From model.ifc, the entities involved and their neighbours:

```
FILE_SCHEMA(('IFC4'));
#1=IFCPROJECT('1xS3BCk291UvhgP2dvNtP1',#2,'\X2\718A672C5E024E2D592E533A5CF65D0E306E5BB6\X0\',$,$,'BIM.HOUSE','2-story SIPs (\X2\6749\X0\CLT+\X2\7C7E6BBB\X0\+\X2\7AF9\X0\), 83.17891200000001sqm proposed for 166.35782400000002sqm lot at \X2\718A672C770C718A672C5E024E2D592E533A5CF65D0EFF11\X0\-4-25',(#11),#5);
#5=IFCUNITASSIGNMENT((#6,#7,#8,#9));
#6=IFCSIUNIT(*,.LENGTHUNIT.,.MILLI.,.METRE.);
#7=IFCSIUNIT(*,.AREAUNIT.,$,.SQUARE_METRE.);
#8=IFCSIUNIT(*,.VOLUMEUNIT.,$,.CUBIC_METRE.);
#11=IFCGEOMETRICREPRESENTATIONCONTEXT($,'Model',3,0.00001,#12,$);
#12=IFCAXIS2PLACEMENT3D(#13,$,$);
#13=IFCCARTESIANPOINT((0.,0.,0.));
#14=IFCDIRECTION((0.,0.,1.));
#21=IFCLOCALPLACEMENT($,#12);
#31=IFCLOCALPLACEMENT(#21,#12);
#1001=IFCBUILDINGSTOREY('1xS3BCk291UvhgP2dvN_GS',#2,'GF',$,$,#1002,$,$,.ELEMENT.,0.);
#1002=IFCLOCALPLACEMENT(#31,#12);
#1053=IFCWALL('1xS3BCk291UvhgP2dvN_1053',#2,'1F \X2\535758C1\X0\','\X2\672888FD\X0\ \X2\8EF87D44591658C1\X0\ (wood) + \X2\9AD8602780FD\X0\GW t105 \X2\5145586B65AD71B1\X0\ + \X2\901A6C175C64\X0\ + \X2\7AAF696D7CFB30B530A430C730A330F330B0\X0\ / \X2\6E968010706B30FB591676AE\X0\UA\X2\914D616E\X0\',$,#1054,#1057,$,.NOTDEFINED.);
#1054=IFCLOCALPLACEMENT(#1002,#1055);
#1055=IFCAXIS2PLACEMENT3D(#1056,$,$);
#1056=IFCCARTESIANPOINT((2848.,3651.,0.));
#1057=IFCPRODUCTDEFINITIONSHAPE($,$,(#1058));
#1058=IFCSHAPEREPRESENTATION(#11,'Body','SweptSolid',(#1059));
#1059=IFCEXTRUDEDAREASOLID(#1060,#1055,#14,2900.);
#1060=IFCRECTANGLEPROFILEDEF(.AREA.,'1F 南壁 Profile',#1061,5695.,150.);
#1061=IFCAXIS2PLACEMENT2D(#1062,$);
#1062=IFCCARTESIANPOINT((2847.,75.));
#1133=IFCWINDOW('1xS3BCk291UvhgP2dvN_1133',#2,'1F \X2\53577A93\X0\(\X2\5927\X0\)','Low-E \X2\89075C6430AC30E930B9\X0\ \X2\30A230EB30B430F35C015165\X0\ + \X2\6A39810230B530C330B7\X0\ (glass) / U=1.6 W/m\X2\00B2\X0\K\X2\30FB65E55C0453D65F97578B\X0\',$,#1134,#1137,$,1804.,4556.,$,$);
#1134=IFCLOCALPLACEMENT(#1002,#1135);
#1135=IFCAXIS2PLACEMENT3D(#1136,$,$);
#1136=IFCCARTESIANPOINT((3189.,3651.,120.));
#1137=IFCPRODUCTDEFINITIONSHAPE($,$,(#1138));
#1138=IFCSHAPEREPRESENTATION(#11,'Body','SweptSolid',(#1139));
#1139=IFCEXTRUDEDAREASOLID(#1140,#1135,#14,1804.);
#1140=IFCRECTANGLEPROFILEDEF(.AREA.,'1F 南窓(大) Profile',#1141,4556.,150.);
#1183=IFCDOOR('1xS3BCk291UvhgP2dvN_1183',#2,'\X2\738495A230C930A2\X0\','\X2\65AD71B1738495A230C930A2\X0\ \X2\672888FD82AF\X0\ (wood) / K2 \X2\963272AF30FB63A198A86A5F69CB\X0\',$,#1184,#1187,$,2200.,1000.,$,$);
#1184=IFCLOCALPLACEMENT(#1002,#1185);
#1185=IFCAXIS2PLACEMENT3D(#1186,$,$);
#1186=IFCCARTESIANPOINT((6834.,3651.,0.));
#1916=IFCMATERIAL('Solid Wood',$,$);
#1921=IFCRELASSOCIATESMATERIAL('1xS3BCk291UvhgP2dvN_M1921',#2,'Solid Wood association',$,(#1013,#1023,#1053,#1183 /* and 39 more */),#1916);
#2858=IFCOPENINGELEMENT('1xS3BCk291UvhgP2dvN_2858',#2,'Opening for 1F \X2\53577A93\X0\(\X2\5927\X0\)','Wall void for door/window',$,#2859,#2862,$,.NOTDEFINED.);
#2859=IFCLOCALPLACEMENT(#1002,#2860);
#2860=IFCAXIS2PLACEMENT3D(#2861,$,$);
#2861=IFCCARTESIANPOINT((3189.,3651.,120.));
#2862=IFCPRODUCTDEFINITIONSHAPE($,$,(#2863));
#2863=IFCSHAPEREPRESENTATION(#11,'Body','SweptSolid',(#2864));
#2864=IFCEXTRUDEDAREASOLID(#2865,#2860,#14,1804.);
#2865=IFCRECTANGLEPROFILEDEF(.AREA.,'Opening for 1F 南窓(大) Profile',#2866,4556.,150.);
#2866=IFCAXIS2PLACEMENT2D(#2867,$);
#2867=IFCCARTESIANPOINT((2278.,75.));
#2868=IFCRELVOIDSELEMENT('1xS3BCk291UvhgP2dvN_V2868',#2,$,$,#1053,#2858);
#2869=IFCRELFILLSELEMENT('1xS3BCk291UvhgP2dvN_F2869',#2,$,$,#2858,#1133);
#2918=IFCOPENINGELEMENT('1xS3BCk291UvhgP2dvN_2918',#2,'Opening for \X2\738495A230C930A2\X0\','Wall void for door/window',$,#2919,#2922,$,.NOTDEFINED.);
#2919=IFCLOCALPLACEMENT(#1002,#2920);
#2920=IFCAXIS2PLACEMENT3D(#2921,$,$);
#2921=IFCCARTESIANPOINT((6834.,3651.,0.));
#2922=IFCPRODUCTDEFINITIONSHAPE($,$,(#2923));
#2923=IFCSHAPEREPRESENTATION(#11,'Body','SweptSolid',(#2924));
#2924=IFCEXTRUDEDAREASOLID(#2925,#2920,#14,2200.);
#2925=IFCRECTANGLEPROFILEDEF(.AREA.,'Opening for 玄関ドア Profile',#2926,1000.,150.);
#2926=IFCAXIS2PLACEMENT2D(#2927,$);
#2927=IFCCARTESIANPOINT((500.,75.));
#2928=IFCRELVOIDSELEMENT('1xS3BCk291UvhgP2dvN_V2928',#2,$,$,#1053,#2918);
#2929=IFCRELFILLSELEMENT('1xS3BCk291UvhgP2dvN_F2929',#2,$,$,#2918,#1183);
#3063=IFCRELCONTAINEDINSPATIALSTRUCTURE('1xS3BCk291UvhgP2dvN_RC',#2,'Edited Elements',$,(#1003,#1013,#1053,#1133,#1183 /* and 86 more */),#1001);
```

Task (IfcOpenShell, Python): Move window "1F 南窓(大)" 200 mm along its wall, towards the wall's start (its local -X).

```python
import ifcopenshell
import ifcopenshell.api.geometry
import ifcopenshell.util.placement
import ifcopenshell.util.unit

model = ifcopenshell.open("model.ifc")
unit_scale = ifcopenshell.util.unit.calculate_unit_scale(model)

window = model.by_guid("1xS3BCk291UvhgP2dvN_1133")
opening = window.FillsVoids[0].RelatingOpeningElement
wall = opening.VoidsElements[0].RelatingBuildingElement

wall_matrix = ifcopenshell.util.placement.get_local_placement(wall.ObjectPlacement)
shift = wall_matrix[:3, 0] * -0.2 / unit_scale
before = ifcopenshell.util.placement.get_local_placement(window.ObjectPlacement)[:3, 3].copy()

# The window is not placed relative to its opening, so move both.
for product in (opening, window):
    matrix = ifcopenshell.util.placement.get_local_placement(product.ObjectPlacement)
    matrix[:3, 3] += shift
    ifcopenshell.api.geometry.edit_object_placement(model, product=product, matrix=matrix, is_si=False)

after = ifcopenshell.util.placement.get_local_placement(window.ObjectPlacement)[:3, 3]
print("window moved by", (after - before).round(3) + 0.0)

model.write("model_v2.ifc")
```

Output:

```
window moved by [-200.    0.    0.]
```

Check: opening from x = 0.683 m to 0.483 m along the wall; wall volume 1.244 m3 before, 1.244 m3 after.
